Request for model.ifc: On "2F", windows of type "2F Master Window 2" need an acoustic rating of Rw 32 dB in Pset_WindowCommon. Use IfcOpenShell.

First a look at what the model holds.

```python
import ifcopenshell
import ifcopenshell.util.element

model = ifcopenshell.open("model.ifc")
print(model.schema)
storey = next(s for s in model.by_type("IfcBuildingStorey") if s.Name == "2F")
windows = [e for e in ifcopenshell.util.element.get_decomposition(storey) if e.is_a("IfcWindow")]
seen = {}
for e in windows:
    element_type = ifcopenshell.util.element.get_type(e)
    key = (element_type.Name if element_type != e and element_type else None, ifcopenshell.util.element.get_pset(e, "Pset_WindowCommon", "AcousticRating"))
    seen[key] = seen.get(key, 0) + 1
for (name, value), count in sorted(seen.items(), key=str):
    print(count, "x", name, "|", value)
```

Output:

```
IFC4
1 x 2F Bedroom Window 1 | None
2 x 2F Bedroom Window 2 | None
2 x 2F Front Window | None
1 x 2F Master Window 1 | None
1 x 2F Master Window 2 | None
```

```python
import ifcopenshell
import ifcopenshell.api.pset
import ifcopenshell.util.element

model = ifcopenshell.open("model.ifc")

storey = next(s for s in model.by_type("IfcBuildingStorey") if s.Name == "2F")
windows = [e for e in ifcopenshell.util.element.get_decomposition(storey) if e.is_a("IfcWindow")]

count = 0
for e in windows:
    element_type = ifcopenshell.util.element.get_type(e)
    if element_type in (None, e) or element_type.Name != "2F Master Window 2":
        continue
    # add_pset returns the element's existing set when there is one.
    pset = ifcopenshell.api.pset.add_pset(model, product=e, name="Pset_WindowCommon")
    ifcopenshell.api.pset.edit_pset(model, pset=pset, properties={"AcousticRating": "Rw 32 dB"})
    count += 1

print(count, "windows updated")

model.write("model_rev.ifc")
```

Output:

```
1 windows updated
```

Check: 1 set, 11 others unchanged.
